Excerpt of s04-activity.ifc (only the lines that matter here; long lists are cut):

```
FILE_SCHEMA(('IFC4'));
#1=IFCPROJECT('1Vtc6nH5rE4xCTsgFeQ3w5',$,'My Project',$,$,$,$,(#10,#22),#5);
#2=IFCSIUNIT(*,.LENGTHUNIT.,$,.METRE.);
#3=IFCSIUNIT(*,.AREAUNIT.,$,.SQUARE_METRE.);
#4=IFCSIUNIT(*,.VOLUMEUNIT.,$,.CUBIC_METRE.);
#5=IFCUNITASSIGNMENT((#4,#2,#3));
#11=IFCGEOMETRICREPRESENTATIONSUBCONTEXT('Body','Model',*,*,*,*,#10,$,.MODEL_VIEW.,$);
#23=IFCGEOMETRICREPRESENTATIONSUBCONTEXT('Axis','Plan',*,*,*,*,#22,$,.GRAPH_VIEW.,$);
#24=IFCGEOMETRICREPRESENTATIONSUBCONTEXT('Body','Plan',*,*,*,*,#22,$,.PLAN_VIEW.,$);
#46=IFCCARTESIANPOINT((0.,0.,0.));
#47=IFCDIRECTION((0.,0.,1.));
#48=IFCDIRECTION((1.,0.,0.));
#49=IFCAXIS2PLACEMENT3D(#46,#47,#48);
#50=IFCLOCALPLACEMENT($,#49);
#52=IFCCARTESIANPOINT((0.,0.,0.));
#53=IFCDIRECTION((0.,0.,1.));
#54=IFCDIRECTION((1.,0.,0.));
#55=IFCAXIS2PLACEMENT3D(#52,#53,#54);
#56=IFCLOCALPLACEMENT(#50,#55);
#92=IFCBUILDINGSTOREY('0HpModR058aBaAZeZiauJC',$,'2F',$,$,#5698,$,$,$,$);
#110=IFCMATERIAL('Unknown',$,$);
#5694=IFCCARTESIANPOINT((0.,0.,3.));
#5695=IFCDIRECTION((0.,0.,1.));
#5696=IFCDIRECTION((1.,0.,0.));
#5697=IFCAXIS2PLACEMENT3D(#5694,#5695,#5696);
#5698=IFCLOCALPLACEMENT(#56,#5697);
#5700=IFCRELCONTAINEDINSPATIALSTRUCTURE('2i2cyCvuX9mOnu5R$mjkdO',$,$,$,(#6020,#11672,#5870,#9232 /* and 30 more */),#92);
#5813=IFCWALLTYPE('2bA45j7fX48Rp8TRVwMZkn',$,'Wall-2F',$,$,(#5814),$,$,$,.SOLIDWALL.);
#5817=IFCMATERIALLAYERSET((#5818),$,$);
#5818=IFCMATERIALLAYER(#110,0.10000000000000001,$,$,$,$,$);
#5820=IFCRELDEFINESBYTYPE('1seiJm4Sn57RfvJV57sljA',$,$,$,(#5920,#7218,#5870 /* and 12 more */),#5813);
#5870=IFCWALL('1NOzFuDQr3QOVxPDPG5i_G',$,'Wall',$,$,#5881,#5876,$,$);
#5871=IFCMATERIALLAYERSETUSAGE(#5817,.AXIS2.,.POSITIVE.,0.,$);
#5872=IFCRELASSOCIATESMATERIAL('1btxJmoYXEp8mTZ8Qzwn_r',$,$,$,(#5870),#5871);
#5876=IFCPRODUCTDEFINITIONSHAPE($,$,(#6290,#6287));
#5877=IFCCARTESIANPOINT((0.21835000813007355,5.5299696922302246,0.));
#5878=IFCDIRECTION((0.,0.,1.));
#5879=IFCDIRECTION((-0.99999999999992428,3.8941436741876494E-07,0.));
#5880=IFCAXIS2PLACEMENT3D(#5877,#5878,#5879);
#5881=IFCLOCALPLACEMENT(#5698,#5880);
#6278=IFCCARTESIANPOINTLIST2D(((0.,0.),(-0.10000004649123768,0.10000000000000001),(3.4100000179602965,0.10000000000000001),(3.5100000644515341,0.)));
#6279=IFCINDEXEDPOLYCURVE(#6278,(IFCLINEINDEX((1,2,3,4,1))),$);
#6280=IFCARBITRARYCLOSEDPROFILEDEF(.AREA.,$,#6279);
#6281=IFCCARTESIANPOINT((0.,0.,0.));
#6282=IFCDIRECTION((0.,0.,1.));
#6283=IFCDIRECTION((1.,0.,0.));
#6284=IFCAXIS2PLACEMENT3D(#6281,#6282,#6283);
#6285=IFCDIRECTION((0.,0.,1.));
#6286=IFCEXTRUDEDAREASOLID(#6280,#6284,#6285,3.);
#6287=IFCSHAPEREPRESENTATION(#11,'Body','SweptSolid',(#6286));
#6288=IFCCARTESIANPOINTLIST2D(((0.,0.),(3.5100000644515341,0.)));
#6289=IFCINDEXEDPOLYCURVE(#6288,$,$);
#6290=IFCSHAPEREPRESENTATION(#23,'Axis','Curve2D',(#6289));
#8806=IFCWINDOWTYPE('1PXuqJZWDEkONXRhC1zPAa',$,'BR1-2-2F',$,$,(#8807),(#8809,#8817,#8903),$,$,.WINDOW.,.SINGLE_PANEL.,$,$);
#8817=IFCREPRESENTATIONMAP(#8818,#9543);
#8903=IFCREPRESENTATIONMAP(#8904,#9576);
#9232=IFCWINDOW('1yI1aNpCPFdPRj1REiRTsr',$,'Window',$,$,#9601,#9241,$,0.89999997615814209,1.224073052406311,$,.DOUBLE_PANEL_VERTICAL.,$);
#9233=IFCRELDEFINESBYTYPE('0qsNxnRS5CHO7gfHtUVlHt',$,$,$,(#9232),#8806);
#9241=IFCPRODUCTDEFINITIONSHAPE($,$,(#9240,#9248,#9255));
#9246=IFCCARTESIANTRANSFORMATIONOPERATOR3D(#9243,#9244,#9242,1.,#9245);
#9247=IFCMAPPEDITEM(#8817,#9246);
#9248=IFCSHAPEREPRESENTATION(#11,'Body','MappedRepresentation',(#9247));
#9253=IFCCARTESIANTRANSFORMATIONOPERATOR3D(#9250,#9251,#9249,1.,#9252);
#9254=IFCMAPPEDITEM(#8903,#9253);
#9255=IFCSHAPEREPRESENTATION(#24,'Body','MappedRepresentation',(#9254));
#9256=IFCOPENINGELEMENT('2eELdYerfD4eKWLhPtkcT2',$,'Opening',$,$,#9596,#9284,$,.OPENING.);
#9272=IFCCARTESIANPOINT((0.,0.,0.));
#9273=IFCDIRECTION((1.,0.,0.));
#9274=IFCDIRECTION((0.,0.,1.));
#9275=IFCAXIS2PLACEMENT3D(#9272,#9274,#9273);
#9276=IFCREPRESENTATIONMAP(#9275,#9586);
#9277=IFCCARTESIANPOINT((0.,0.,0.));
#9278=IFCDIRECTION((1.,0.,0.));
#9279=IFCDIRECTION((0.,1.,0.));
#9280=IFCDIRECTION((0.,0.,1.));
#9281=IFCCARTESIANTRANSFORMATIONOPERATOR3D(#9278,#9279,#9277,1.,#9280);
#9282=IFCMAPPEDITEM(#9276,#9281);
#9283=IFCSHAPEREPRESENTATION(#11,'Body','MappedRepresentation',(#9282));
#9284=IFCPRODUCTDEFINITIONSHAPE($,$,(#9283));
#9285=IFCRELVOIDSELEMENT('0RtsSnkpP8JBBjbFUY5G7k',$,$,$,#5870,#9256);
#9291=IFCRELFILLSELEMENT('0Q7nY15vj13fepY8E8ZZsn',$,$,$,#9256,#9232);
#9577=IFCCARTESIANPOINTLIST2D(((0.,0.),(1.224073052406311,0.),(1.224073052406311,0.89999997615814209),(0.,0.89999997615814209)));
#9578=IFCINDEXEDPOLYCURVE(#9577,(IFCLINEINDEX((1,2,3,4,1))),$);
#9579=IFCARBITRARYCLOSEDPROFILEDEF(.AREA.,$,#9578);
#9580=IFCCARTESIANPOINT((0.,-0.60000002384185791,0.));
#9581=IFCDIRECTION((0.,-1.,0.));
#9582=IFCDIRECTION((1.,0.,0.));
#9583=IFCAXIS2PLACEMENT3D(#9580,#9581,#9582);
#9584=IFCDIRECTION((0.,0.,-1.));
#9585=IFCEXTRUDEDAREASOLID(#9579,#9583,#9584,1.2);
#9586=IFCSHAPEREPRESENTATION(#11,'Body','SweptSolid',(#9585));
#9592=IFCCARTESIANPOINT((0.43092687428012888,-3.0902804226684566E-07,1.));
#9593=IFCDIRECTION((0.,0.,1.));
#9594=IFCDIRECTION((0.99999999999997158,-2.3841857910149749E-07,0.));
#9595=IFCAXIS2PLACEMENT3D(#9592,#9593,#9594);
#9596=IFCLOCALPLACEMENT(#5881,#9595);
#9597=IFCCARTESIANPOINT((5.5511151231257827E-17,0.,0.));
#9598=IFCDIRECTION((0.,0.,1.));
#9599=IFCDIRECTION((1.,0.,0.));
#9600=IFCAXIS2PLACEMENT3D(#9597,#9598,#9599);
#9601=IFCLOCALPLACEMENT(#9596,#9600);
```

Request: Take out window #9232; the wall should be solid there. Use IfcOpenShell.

```python
import ifcopenshell
import ifcopenshell.api.feature
import ifcopenshell.api.root
import ifcopenshell.geom
import ifcopenshell.util.shape

model = ifcopenshell.open("s04-activity.ifc")
settings = ifcopenshell.geom.settings()


def volume(element):
    """Net volume in cubic metres, openings subtracted."""
    shape = ifcopenshell.geom.create_shape(settings, element)
    return ifcopenshell.util.shape.get_volume(shape.geometry)


window = model.by_guid("1yI1aNpCPFdPRj1REiRTsr")
opening = window.FillsVoids[0].RelatingOpeningElement
wall = opening.VoidsElements[0].RelatingBuildingElement
before = volume(wall)

ifcopenshell.api.root.remove_product(model, product=window)
ifcopenshell.api.feature.remove_feature(model, feature=opening)

after = volume(wall)

print(f"wall volume {before:.3f} -> {after:.3f} m3")

model.write("s04-activity_updated.ifc")
```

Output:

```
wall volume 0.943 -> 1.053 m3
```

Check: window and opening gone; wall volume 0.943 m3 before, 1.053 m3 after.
